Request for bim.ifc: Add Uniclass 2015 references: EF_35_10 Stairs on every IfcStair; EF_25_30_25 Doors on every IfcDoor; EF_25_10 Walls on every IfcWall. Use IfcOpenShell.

First a look at what the model holds.

```python
import ifcopenshell

model = ifcopenshell.open("bim.ifc")
print(model.schema)
print("classifications:", [c.Name for c in model.by_type("IfcClassification")])
for ifc_class in ("IfcDoor", "IfcRoof", "IfcStair", "IfcWall", "IfcWindow"):
    print(ifc_class, len(model.by_type(ifc_class)))
```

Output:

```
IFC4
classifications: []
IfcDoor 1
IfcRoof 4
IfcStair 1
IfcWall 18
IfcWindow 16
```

```python
import ifcopenshell
import ifcopenshell.api.classification

model = ifcopenshell.open("bim.ifc")

system = ifcopenshell.api.classification.add_classification(model, classification="Uniclass 2015")

codes = {
    "IfcStair": ("EF_35_10", "Stairs"),
    "IfcDoor": ("EF_25_30_25", "Doors"),
    "IfcWall": ("EF_25_10", "Walls"),
}
for ifc_class, (code, name) in codes.items():
    products = model.by_type(ifc_class)
    ifcopenshell.api.classification.add_reference(
        model, products=products, classification=system, identification=code, name=name
    )
    print(code, len(products))

model.write("bim-out.ifc")
```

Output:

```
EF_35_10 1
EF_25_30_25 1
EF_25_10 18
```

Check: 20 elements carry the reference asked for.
